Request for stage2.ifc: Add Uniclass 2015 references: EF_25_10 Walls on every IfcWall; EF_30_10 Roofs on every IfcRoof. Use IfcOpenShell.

First a look at what the model holds.

```python
import ifcopenshell

model = ifcopenshell.open("stage2.ifc")
print(model.schema)
print("classifications:", [c.Name for c in model.by_type("IfcClassification")])
for ifc_class in ("IfcDoor", "IfcRoof", "IfcStair", "IfcWall", "IfcWindow"):
    print(ifc_class, len(model.by_type(ifc_class)))
```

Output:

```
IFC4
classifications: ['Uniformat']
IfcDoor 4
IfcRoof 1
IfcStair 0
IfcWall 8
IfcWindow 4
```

```python
import ifcopenshell
import ifcopenshell.api.classification

model = ifcopenshell.open("stage2.ifc")

system = ifcopenshell.api.classification.add_classification(model, classification="Uniclass 2015")

codes = {
    "IfcWall": ("EF_25_10", "Walls"),
    "IfcRoof": ("EF_30_10", "Roofs"),
}
for ifc_class, (code, name) in codes.items():
    products = model.by_type(ifc_class)
    ifcopenshell.api.classification.add_reference(
        model, products=products, classification=system, identification=code, name=name
    )
    print(code, len(products))

model.write("stage2_v2.ifc")
```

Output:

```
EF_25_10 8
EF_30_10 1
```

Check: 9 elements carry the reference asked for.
